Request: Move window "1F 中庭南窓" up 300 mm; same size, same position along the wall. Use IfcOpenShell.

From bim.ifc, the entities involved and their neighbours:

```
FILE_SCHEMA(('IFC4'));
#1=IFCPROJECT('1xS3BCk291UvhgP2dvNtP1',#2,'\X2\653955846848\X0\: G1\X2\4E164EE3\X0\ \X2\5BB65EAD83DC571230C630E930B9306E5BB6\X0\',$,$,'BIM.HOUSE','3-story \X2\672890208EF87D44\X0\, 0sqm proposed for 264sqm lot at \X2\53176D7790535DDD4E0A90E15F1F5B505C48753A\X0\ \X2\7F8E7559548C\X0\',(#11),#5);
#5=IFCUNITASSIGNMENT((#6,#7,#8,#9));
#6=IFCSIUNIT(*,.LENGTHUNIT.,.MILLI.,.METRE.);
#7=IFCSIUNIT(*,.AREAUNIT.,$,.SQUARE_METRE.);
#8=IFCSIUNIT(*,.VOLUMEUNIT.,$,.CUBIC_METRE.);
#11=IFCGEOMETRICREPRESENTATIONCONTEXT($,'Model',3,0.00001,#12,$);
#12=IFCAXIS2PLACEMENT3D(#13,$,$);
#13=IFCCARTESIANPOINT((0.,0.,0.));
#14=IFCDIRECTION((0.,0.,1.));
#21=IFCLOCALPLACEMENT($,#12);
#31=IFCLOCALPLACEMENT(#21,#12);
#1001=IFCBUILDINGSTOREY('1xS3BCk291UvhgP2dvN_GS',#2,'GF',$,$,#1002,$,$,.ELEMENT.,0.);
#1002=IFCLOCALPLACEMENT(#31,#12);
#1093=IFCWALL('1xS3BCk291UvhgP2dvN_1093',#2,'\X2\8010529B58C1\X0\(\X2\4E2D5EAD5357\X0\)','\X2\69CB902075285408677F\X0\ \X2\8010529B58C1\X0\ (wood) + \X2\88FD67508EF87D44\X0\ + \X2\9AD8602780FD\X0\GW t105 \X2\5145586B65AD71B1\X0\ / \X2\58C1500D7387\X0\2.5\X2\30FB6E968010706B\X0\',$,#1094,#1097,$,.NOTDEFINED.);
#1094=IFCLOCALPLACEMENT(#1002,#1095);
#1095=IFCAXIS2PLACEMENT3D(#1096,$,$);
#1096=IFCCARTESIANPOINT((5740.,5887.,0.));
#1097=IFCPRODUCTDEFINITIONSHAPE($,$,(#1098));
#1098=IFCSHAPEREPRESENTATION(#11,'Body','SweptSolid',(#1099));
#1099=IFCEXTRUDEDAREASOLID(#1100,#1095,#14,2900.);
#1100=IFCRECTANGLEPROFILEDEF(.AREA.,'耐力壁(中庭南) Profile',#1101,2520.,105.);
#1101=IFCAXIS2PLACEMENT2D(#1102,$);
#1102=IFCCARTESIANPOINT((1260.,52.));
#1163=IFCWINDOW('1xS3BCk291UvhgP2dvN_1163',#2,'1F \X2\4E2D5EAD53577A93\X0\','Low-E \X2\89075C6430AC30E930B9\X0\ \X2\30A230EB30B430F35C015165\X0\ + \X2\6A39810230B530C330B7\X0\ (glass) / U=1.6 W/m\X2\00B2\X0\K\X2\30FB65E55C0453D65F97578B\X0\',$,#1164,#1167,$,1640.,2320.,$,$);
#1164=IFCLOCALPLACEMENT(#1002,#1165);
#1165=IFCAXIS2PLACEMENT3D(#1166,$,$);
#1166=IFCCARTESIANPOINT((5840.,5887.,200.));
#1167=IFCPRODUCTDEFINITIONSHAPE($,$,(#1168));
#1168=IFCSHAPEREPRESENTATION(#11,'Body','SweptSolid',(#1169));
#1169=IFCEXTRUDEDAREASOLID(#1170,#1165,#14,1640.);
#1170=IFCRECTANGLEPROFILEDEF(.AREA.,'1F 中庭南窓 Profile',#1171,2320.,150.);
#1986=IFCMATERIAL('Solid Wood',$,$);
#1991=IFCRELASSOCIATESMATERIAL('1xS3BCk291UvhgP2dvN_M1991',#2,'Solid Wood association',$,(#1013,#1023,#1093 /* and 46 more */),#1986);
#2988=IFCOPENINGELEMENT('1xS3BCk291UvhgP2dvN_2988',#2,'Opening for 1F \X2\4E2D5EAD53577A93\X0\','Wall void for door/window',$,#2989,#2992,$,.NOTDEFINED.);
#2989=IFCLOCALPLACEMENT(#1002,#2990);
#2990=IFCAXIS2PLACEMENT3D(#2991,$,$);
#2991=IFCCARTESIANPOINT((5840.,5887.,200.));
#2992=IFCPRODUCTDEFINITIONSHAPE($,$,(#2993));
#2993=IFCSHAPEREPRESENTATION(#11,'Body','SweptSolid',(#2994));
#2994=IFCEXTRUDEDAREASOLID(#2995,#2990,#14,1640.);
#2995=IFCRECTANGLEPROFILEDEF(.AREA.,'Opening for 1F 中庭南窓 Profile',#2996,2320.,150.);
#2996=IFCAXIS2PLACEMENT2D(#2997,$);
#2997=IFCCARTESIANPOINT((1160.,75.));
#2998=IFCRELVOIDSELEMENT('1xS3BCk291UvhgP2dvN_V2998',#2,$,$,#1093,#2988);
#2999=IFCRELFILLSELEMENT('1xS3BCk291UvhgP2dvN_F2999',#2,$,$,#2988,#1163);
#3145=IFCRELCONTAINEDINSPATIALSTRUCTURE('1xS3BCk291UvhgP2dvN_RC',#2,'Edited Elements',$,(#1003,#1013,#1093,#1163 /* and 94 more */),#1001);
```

```python
import numpy as np
import ifcopenshell
import ifcopenshell.api.geometry
import ifcopenshell.util.placement
import ifcopenshell.util.unit

model = ifcopenshell.open("bim.ifc")
unit_scale = ifcopenshell.util.unit.calculate_unit_scale(model)

window = model.by_guid("1xS3BCk291UvhgP2dvN_1163")
opening = window.FillsVoids[0].RelatingOpeningElement
dz = 0.3 / unit_scale

shift = np.array([0.0, 0.0, dz])
# The window is not placed relative to its opening, so move both.
for product in (opening, window):
    matrix = ifcopenshell.util.placement.get_local_placement(product.ObjectPlacement)
    matrix[:3, 3] += shift
    ifcopenshell.api.geometry.edit_object_placement(model, product=product, matrix=matrix, is_si=False)

print(f"moved by {dz * unit_scale:+.3f} m")

model.write("bim_updated.ifc")
```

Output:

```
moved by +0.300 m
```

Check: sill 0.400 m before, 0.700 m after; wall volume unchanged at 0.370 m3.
